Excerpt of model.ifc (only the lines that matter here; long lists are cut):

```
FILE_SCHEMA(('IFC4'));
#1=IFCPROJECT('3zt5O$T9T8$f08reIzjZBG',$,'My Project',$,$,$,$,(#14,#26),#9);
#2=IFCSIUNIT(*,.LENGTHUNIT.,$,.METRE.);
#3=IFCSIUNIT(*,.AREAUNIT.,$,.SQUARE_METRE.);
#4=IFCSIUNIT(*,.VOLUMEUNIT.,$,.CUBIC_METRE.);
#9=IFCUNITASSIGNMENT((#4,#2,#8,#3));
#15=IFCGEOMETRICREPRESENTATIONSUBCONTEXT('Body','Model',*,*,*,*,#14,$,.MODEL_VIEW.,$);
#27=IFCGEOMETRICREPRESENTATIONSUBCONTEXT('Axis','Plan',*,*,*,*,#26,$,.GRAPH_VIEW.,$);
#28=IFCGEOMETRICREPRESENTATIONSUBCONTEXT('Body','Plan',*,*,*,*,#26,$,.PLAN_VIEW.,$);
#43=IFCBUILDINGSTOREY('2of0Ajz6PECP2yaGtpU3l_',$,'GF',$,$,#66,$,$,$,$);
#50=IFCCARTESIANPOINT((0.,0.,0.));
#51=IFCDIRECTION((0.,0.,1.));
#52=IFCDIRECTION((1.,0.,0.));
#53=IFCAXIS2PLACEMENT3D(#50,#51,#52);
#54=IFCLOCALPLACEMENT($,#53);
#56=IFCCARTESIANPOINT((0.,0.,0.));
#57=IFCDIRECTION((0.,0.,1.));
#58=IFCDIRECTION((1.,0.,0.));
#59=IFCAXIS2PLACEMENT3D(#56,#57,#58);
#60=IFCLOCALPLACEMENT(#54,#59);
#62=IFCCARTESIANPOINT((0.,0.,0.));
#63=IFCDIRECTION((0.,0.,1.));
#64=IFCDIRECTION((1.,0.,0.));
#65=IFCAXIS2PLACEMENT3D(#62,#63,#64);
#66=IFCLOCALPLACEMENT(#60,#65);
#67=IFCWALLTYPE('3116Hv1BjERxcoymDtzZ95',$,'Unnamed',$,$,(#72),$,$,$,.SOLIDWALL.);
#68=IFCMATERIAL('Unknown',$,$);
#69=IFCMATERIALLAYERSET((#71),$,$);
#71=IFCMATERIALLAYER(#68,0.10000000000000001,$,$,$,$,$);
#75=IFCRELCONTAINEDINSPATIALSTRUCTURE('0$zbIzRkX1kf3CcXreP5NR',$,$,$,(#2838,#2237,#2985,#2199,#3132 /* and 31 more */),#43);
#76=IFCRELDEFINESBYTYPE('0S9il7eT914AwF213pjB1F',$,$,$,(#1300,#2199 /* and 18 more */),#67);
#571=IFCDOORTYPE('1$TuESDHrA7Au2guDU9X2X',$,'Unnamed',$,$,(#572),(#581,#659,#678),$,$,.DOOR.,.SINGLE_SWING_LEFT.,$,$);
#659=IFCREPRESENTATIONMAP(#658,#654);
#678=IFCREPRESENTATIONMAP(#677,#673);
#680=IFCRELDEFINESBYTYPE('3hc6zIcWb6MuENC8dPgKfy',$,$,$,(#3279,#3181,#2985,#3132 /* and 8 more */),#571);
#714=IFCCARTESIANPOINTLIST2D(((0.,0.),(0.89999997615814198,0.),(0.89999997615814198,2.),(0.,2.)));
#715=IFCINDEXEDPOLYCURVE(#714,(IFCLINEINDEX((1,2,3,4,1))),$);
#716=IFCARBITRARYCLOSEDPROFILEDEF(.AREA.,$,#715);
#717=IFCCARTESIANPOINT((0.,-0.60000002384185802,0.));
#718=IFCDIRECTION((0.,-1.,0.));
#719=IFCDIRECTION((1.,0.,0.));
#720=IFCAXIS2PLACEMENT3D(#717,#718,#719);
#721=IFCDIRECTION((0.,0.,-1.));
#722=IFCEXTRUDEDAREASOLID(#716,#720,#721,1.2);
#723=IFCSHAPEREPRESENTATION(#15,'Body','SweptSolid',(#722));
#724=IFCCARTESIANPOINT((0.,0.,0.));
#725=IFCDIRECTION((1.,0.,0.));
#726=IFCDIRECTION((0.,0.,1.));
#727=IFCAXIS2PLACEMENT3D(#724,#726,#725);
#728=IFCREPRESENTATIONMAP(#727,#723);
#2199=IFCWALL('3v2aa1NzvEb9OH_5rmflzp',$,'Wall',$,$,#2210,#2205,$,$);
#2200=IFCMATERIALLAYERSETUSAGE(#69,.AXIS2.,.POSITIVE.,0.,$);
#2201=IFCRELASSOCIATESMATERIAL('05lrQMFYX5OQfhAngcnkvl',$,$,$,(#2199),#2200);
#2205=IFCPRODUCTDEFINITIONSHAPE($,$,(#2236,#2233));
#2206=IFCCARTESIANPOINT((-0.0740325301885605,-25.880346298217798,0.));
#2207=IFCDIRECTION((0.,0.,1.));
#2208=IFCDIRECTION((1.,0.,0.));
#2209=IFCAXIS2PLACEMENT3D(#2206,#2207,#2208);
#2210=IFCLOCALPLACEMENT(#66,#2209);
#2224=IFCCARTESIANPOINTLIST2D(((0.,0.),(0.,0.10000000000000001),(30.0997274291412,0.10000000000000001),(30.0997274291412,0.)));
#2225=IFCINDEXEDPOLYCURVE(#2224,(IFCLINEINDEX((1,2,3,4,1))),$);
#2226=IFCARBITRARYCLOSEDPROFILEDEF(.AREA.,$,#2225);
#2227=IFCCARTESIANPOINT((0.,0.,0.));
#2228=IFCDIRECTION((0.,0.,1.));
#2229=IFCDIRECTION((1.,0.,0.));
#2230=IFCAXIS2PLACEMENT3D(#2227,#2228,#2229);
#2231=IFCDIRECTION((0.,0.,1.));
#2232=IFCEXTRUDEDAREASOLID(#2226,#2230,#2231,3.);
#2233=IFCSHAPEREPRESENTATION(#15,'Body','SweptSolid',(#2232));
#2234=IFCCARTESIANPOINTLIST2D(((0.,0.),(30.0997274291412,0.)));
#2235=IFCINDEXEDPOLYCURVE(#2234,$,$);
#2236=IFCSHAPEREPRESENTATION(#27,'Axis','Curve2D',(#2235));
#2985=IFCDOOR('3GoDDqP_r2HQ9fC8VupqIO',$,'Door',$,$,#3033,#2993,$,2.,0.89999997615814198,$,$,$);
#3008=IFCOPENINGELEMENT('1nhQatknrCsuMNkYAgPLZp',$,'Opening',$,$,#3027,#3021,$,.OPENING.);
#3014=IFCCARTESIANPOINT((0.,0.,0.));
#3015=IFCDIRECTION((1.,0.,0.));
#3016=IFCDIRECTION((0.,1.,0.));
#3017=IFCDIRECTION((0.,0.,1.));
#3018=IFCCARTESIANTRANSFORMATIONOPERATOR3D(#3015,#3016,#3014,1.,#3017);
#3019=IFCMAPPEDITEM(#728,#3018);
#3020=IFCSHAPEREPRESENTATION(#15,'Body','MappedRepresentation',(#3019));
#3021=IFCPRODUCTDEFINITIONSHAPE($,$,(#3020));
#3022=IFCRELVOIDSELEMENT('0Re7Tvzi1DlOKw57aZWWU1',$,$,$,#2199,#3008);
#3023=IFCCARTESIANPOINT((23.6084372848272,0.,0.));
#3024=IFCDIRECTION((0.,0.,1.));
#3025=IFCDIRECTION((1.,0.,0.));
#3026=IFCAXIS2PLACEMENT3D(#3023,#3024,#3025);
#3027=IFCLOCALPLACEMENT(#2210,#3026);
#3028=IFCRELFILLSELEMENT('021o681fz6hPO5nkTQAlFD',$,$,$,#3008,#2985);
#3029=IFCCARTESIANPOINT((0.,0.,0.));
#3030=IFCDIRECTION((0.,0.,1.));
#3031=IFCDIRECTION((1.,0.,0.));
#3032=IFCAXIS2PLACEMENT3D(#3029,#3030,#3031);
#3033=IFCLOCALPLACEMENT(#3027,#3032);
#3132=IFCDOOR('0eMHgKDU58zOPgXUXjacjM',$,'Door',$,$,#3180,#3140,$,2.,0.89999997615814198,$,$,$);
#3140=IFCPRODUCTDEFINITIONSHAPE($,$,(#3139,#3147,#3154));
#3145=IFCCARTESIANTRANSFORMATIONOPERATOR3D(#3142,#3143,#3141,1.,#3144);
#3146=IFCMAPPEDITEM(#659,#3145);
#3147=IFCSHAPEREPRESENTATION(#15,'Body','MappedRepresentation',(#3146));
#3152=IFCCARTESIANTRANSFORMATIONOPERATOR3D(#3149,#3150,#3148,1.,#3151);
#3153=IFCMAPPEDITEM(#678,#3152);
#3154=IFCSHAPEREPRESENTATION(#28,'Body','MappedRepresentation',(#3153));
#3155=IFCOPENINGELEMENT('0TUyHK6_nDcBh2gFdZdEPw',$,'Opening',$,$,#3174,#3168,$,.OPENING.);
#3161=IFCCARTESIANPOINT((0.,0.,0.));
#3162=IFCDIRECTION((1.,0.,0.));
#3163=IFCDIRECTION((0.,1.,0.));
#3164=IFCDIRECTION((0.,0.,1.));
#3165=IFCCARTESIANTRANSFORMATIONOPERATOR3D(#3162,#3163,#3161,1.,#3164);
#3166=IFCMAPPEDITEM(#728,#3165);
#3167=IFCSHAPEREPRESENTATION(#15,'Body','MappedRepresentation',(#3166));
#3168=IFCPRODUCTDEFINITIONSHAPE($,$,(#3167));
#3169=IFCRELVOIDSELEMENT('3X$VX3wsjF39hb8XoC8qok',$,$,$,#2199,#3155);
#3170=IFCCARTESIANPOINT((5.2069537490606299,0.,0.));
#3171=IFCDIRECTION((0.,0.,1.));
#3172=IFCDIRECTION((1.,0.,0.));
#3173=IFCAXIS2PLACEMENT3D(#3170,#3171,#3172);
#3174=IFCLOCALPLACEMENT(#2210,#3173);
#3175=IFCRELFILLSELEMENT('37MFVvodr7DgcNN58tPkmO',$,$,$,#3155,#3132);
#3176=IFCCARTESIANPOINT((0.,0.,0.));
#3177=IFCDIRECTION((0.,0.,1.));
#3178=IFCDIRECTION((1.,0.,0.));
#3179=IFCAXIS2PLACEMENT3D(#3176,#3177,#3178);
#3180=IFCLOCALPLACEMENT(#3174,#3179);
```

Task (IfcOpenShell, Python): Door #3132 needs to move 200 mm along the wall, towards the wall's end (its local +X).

```python
import ifcopenshell
import ifcopenshell.api.geometry
import ifcopenshell.util.placement
import ifcopenshell.util.unit

model = ifcopenshell.open("model.ifc")
unit_scale = ifcopenshell.util.unit.calculate_unit_scale(model)

door = model.by_guid("0eMHgKDU58zOPgXUXjacjM")
opening = door.FillsVoids[0].RelatingOpeningElement
wall = opening.VoidsElements[0].RelatingBuildingElement

wall_matrix = ifcopenshell.util.placement.get_local_placement(wall.ObjectPlacement)
shift = wall_matrix[:3, 0] * 0.2 / unit_scale
before = ifcopenshell.util.placement.get_local_placement(door.ObjectPlacement)[:3, 3].copy()

# The door is placed relative to its opening, so it follows when the opening moves.
matrix = ifcopenshell.util.placement.get_local_placement(opening.ObjectPlacement)
matrix[:3, 3] += shift
ifcopenshell.api.geometry.edit_object_placement(
    model, product=opening, matrix=matrix, is_si=False, should_transform_children=True
)

after = ifcopenshell.util.placement.get_local_placement(door.ObjectPlacement)[:3, 3]
print("door moved by", (after - before).round(3) + 0.0)

model.write("model_v2.ifc")
```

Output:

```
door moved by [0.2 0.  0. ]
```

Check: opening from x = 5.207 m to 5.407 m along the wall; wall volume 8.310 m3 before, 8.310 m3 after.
